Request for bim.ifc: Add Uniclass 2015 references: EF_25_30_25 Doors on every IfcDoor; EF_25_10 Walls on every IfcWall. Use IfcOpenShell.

First a look at what the model holds.

```python
import ifcopenshell

model = ifcopenshell.open("bim.ifc")
print(model.schema)
print("classifications:", [c.Name for c in model.by_type("IfcClassification")])
for ifc_class in ("IfcDoor", "IfcRoof", "IfcStair", "IfcWall", "IfcWindow"):
    print(ifc_class, len(model.by_type(ifc_class)))
```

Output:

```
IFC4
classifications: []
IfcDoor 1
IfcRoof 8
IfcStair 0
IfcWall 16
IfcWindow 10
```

```python
import ifcopenshell
import ifcopenshell.api.classification

model = ifcopenshell.open("bim.ifc")

system = ifcopenshell.api.classification.add_classification(model, classification="Uniclass 2015")

codes = {
    "IfcDoor": ("EF_25_30_25", "Doors"),
    "IfcWall": ("EF_25_10", "Walls"),
}
for ifc_class, (code, name) in codes.items():
    products = model.by_type(ifc_class)
    ifcopenshell.api.classification.add_reference(
        model, products=products, classification=system, identification=code, name=name
    )
    print(code, len(products))

model.write("bim_v2.ifc")
```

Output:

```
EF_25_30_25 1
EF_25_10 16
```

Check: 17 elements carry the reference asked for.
